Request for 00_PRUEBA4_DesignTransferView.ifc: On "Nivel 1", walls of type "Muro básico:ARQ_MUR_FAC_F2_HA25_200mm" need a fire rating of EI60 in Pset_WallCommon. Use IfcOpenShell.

First a look at what the model holds.

```python
import ifcopenshell
import ifcopenshell.util.element

model = ifcopenshell.open("00_PRUEBA4_DesignTransferView.ifc")
print(model.schema)
storey = next(s for s in model.by_type("IfcBuildingStorey") if s.Name == "Nivel 1")
walls = [e for e in ifcopenshell.util.element.get_decomposition(storey) if e.is_a("IfcWall")]
seen = {}
for e in walls:
    element_type = ifcopenshell.util.element.get_type(e)
    key = (element_type.Name if element_type != e and element_type else None, ifcopenshell.util.element.get_pset(e, "Pset_WallCommon", "FireRating"))
    seen[key] = seen.get(key, 0) + 1
for (name, value), count in sorted(seen.items(), key=str):
    print(count, "x", name, "|", value)
```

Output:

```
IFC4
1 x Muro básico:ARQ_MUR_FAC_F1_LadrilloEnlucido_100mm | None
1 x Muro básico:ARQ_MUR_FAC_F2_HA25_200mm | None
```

```python
import ifcopenshell
import ifcopenshell.api.pset
import ifcopenshell.util.element

model = ifcopenshell.open("00_PRUEBA4_DesignTransferView.ifc")

storey = next(s for s in model.by_type("IfcBuildingStorey") if s.Name == "Nivel 1")
walls = [e for e in ifcopenshell.util.element.get_decomposition(storey) if e.is_a("IfcWall")]

count = 0
for e in walls:
    element_type = ifcopenshell.util.element.get_type(e)
    if element_type in (None, e) or element_type.Name != "Muro básico:ARQ_MUR_FAC_F2_HA25_200mm":
        continue
    # add_pset returns the element's existing set when there is one.
    pset = ifcopenshell.api.pset.add_pset(model, product=e, name="Pset_WallCommon")
    ifcopenshell.api.pset.edit_pset(model, pset=pset, properties={"FireRating": "EI60"})
    count += 1

print(count, "walls updated")

model.write("00_PRUEBA4_DesignTransferView_rev.ifc")
```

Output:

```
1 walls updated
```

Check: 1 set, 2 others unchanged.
